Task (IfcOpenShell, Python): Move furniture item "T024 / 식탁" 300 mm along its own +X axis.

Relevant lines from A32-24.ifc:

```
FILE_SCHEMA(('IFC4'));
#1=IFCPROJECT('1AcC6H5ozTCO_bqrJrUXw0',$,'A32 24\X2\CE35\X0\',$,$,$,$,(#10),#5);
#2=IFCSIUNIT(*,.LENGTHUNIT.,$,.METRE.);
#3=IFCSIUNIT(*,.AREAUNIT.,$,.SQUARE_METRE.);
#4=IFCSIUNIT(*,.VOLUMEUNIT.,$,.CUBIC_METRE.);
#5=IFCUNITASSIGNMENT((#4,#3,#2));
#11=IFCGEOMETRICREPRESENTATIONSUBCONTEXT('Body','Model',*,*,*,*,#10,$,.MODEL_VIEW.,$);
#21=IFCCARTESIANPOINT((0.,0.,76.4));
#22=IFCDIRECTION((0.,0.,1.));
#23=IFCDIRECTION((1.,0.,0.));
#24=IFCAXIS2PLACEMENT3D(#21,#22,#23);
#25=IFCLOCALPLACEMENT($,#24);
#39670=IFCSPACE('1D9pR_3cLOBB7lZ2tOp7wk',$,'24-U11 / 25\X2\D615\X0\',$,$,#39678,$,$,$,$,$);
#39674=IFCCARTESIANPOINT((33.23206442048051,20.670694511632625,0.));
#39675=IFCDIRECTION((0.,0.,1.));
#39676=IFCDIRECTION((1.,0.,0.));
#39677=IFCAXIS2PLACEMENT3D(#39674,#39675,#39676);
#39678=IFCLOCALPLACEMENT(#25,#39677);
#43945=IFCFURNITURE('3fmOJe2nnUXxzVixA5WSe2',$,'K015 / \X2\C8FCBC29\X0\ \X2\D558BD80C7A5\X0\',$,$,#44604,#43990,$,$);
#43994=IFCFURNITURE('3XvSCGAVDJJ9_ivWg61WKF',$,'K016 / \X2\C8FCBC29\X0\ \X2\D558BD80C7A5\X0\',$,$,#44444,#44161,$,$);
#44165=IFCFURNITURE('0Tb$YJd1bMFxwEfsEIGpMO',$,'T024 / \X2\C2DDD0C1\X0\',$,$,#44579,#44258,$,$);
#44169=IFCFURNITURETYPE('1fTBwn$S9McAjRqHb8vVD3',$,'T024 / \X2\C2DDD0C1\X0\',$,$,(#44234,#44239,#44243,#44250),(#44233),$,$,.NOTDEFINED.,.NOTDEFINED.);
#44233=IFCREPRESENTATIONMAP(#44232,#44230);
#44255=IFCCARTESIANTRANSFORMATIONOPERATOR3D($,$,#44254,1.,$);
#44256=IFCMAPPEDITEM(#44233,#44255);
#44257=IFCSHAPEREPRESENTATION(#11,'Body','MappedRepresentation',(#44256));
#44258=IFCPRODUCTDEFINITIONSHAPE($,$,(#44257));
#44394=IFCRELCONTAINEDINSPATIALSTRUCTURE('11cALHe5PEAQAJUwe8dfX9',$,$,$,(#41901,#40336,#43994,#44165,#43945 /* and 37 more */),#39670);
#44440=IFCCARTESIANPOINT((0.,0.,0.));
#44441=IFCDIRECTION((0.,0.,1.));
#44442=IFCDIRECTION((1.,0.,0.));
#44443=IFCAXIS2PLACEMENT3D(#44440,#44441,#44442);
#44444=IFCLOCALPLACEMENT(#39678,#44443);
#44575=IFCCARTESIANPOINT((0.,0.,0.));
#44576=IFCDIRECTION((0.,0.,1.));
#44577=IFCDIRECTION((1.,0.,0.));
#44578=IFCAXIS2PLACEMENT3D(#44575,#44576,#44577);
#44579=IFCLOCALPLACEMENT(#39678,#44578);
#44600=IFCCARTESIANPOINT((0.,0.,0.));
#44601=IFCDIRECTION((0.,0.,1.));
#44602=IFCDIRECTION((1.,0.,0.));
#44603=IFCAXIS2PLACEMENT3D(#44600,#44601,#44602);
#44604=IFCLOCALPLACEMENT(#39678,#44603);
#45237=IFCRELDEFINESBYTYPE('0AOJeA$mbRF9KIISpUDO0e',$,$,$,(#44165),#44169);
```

```python
import ifcopenshell
import ifcopenshell.api.geometry
import ifcopenshell.util.placement
import ifcopenshell.util.unit

model = ifcopenshell.open("A32-24.ifc")
unit_scale = ifcopenshell.util.unit.calculate_unit_scale(model)

item = model.by_id(44165)
matrix = ifcopenshell.util.placement.get_local_placement(item.ObjectPlacement)
matrix[:3, 3] += matrix[:3, 0] * 0.3 / unit_scale
ifcopenshell.api.geometry.edit_object_placement(model, product=item, matrix=matrix, is_si=False)

print(ifcopenshell.util.placement.get_local_placement(item.ObjectPlacement).round(3) + 0.0)

model.write("A32-24_updated.ifc")
```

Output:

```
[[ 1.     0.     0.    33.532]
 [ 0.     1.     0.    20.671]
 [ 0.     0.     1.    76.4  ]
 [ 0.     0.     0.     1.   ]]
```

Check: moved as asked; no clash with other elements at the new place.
